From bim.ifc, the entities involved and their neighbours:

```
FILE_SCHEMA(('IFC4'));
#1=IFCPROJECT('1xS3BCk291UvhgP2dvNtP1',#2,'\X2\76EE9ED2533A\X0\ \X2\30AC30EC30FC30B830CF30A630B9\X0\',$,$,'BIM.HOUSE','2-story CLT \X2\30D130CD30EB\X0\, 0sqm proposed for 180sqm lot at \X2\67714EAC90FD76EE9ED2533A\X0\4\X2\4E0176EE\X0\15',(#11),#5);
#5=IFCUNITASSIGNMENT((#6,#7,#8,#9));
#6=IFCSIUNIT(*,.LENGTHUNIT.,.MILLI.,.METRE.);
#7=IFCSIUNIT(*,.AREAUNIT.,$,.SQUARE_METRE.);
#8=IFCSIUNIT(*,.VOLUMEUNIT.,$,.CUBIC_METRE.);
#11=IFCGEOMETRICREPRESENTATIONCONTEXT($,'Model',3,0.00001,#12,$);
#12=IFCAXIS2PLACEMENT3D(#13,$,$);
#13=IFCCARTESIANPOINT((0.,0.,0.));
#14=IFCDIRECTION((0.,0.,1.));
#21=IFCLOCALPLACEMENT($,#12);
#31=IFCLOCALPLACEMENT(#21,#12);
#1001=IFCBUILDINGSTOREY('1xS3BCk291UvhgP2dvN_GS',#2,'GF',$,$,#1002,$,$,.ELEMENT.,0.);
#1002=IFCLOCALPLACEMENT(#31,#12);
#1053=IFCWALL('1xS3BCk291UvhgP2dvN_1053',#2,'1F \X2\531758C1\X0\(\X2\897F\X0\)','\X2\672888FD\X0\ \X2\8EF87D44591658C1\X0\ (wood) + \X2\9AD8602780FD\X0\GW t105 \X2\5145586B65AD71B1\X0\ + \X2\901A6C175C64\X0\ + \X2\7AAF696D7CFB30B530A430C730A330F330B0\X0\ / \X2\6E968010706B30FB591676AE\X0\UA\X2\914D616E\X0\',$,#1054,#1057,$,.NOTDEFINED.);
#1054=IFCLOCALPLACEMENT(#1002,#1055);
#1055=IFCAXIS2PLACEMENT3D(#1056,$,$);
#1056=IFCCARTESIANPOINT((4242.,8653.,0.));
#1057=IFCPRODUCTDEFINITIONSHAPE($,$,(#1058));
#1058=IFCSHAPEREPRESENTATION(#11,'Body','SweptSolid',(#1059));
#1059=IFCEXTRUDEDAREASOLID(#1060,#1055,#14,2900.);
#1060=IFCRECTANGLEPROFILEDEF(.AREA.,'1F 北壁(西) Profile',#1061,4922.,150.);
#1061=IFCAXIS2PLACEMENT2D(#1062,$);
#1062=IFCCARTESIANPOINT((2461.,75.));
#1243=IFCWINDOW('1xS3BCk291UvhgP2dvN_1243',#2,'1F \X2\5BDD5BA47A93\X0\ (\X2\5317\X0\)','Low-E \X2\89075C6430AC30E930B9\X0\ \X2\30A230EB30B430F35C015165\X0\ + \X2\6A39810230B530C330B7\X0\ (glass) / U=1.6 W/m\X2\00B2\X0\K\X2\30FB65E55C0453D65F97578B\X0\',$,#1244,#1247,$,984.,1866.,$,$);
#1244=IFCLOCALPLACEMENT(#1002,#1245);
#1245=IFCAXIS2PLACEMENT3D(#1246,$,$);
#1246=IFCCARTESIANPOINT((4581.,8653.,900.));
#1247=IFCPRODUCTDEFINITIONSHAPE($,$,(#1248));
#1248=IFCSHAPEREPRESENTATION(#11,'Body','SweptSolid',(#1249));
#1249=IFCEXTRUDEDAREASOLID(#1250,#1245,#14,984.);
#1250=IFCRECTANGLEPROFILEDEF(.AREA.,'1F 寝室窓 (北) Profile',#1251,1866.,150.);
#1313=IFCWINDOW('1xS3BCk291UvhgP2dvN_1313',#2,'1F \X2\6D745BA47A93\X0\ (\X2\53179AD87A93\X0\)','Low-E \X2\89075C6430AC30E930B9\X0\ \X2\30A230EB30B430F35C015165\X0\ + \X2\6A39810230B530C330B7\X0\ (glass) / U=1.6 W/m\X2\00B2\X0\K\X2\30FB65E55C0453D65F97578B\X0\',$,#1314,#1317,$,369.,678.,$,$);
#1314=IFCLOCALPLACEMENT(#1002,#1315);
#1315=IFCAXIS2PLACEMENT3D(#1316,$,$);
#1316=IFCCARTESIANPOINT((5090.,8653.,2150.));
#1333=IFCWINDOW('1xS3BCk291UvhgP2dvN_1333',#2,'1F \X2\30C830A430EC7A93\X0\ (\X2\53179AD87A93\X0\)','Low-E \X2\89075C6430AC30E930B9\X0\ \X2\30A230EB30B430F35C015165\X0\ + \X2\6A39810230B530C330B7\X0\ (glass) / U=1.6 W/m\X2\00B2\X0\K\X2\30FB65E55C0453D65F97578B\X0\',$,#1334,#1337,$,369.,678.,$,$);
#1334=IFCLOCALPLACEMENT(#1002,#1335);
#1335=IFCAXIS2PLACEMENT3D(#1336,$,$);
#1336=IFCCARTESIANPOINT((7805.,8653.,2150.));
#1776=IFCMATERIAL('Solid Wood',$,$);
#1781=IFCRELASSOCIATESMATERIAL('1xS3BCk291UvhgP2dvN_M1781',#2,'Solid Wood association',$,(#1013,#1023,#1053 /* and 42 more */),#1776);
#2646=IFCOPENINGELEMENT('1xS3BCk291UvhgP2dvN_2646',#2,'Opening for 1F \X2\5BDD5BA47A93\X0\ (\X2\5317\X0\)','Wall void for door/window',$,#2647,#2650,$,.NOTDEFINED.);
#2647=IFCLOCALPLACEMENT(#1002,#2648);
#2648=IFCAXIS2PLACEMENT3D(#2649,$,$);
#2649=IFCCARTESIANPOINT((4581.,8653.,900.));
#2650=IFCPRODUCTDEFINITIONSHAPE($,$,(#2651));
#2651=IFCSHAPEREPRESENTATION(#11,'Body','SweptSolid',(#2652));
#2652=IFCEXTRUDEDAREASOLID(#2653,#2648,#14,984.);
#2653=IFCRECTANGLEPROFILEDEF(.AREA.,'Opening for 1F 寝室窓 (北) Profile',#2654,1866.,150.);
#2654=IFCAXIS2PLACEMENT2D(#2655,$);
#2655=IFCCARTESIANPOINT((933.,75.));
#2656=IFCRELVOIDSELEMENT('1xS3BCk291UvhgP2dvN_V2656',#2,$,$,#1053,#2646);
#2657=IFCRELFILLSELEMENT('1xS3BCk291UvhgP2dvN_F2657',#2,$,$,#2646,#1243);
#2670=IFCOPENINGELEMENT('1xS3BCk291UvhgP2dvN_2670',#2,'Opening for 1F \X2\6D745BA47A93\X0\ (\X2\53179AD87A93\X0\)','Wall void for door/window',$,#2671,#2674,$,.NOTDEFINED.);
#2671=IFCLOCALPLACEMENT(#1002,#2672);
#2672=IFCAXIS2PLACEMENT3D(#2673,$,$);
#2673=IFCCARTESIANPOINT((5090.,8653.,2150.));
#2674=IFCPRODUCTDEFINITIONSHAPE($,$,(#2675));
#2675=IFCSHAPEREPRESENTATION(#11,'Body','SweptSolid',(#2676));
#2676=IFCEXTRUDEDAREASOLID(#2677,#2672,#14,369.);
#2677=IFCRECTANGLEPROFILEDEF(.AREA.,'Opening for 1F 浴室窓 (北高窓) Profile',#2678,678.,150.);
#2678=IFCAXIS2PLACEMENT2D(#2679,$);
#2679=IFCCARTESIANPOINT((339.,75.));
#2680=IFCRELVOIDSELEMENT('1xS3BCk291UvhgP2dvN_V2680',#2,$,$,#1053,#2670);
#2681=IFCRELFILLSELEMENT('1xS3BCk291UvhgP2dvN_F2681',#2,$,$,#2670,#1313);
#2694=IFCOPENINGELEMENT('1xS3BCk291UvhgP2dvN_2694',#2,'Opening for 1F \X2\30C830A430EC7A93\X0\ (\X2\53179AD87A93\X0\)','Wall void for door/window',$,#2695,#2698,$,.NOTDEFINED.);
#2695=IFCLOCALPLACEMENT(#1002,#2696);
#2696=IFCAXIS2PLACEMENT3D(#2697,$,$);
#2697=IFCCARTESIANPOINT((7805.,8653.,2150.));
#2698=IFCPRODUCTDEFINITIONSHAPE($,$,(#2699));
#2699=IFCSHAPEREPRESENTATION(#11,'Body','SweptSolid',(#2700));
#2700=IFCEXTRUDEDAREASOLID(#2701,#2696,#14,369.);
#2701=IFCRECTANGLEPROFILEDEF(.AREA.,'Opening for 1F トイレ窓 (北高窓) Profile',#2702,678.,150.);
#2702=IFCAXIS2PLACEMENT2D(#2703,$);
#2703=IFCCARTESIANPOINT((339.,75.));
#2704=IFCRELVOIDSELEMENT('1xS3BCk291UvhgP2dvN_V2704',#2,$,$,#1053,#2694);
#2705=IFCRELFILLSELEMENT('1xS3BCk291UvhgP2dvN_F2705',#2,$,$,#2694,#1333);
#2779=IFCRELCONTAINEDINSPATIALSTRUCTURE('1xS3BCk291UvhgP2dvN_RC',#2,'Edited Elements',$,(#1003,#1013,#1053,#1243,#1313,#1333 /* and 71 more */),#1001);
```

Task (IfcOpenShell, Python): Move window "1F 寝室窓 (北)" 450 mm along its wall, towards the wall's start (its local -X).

```python
import ifcopenshell
import ifcopenshell.api.geometry
import ifcopenshell.util.placement
import ifcopenshell.util.unit

model = ifcopenshell.open("bim.ifc")
unit_scale = ifcopenshell.util.unit.calculate_unit_scale(model)

window = model.by_guid("1xS3BCk291UvhgP2dvN_1243")
opening = window.FillsVoids[0].RelatingOpeningElement
wall = opening.VoidsElements[0].RelatingBuildingElement

wall_matrix = ifcopenshell.util.placement.get_local_placement(wall.ObjectPlacement)
shift = wall_matrix[:3, 0] * -0.45 / unit_scale
before = ifcopenshell.util.placement.get_local_placement(window.ObjectPlacement)[:3, 3].copy()

# The window is not placed relative to its opening, so move both.
for product in (opening, window):
    matrix = ifcopenshell.util.placement.get_local_placement(product.ObjectPlacement)
    matrix[:3, 3] += shift
    ifcopenshell.api.geometry.edit_object_placement(model, product=product, matrix=matrix, is_si=False)

after = ifcopenshell.util.placement.get_local_placement(window.ObjectPlacement)[:3, 3]
print("window moved by", (after - before).round(3) + 0.0)

model.write("bim_v2.ifc")
```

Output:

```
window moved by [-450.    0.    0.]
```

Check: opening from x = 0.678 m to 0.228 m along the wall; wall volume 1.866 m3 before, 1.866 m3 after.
